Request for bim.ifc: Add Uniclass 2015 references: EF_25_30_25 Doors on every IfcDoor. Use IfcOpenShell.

First a look at what the model holds.

```python
import ifcopenshell

model = ifcopenshell.open("bim.ifc")
print(model.schema)
print("classifications:", [c.Name for c in model.by_type("IfcClassification")])
for ifc_class in ("IfcDoor", "IfcRoof", "IfcStair", "IfcWall", "IfcWindow"):
    print(ifc_class, len(model.by_type(ifc_class)))
```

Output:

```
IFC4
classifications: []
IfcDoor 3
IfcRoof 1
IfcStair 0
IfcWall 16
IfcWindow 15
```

```python
import ifcopenshell
import ifcopenshell.api.classification

model = ifcopenshell.open("bim.ifc")

system = ifcopenshell.api.classification.add_classification(model, classification="Uniclass 2015")

codes = {
    "IfcDoor": ("EF_25_30_25", "Doors"),
}
for ifc_class, (code, name) in codes.items():
    products = model.by_type(ifc_class)
    ifcopenshell.api.classification.add_reference(
        model, products=products, classification=system, identification=code, name=name
    )
    print(code, len(products))

model.write("bim_rev.ifc")
```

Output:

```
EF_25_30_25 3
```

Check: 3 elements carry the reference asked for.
